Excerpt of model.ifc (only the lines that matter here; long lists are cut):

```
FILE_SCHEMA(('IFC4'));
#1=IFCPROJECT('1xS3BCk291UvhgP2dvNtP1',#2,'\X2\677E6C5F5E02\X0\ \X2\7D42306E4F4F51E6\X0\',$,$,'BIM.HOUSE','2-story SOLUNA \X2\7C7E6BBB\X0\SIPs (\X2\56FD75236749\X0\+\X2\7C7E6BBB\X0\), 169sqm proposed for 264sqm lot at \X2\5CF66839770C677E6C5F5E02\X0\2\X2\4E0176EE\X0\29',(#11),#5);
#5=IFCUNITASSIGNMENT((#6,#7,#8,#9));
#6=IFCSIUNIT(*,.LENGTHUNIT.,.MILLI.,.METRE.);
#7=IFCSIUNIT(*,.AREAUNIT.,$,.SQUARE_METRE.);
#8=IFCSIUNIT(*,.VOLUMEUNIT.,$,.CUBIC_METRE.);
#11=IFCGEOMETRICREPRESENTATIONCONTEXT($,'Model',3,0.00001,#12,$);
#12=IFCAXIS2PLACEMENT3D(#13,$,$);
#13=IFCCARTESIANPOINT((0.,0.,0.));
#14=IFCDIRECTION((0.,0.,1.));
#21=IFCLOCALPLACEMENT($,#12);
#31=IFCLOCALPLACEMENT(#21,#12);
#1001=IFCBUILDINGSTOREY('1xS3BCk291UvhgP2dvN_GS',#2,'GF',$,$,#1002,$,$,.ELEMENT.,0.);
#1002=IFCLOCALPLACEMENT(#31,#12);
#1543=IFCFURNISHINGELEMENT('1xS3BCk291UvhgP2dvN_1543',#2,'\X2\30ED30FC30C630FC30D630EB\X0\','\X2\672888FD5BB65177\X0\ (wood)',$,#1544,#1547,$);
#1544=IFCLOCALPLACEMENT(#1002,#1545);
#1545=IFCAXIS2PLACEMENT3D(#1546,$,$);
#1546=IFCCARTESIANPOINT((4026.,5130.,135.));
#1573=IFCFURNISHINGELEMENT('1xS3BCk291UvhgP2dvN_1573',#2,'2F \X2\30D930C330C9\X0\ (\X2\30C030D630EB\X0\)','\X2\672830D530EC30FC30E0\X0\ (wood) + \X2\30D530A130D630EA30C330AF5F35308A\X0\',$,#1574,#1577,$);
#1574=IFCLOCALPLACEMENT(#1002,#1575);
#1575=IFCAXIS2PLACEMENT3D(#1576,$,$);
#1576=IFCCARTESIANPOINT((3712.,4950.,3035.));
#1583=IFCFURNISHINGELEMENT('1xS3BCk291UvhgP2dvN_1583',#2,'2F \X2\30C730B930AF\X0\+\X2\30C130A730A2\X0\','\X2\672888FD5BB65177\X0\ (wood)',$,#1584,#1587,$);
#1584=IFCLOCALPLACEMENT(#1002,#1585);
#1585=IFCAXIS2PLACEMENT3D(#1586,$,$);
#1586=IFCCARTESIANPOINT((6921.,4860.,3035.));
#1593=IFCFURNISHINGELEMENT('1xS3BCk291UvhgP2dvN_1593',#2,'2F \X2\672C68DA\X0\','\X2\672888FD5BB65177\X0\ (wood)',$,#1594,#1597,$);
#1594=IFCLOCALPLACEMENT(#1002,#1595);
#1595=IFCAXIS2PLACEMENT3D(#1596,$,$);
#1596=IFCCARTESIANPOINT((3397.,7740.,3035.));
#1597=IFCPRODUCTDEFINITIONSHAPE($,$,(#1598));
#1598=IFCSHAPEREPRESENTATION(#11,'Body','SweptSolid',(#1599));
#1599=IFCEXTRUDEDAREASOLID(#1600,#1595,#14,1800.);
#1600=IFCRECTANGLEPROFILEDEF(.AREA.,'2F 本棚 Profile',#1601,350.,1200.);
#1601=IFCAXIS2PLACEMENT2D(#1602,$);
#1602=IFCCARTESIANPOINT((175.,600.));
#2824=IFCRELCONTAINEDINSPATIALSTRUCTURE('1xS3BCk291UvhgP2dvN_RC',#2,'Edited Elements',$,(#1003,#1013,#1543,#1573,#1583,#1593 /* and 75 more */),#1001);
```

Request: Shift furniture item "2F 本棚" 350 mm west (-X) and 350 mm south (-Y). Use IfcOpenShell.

```python
import ifcopenshell
import ifcopenshell.api.geometry
import ifcopenshell.util.placement

model = ifcopenshell.open("model.ifc")

item = model.by_guid("1xS3BCk291UvhgP2dvN_1593")
matrix = ifcopenshell.util.placement.get_local_placement(item.ObjectPlacement)
matrix[0, 3] -= 350.0
matrix[1, 3] -= 350.0
ifcopenshell.api.geometry.edit_object_placement(model, product=item, matrix=matrix, is_si=False)

print(ifcopenshell.util.placement.get_local_placement(item.ObjectPlacement).round(3) + 0.0)

model.write("model_v2.ifc")
```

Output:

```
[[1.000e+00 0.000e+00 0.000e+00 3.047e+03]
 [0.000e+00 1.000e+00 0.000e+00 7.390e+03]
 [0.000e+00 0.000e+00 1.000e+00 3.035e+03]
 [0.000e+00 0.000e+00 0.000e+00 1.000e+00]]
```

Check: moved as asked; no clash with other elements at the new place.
